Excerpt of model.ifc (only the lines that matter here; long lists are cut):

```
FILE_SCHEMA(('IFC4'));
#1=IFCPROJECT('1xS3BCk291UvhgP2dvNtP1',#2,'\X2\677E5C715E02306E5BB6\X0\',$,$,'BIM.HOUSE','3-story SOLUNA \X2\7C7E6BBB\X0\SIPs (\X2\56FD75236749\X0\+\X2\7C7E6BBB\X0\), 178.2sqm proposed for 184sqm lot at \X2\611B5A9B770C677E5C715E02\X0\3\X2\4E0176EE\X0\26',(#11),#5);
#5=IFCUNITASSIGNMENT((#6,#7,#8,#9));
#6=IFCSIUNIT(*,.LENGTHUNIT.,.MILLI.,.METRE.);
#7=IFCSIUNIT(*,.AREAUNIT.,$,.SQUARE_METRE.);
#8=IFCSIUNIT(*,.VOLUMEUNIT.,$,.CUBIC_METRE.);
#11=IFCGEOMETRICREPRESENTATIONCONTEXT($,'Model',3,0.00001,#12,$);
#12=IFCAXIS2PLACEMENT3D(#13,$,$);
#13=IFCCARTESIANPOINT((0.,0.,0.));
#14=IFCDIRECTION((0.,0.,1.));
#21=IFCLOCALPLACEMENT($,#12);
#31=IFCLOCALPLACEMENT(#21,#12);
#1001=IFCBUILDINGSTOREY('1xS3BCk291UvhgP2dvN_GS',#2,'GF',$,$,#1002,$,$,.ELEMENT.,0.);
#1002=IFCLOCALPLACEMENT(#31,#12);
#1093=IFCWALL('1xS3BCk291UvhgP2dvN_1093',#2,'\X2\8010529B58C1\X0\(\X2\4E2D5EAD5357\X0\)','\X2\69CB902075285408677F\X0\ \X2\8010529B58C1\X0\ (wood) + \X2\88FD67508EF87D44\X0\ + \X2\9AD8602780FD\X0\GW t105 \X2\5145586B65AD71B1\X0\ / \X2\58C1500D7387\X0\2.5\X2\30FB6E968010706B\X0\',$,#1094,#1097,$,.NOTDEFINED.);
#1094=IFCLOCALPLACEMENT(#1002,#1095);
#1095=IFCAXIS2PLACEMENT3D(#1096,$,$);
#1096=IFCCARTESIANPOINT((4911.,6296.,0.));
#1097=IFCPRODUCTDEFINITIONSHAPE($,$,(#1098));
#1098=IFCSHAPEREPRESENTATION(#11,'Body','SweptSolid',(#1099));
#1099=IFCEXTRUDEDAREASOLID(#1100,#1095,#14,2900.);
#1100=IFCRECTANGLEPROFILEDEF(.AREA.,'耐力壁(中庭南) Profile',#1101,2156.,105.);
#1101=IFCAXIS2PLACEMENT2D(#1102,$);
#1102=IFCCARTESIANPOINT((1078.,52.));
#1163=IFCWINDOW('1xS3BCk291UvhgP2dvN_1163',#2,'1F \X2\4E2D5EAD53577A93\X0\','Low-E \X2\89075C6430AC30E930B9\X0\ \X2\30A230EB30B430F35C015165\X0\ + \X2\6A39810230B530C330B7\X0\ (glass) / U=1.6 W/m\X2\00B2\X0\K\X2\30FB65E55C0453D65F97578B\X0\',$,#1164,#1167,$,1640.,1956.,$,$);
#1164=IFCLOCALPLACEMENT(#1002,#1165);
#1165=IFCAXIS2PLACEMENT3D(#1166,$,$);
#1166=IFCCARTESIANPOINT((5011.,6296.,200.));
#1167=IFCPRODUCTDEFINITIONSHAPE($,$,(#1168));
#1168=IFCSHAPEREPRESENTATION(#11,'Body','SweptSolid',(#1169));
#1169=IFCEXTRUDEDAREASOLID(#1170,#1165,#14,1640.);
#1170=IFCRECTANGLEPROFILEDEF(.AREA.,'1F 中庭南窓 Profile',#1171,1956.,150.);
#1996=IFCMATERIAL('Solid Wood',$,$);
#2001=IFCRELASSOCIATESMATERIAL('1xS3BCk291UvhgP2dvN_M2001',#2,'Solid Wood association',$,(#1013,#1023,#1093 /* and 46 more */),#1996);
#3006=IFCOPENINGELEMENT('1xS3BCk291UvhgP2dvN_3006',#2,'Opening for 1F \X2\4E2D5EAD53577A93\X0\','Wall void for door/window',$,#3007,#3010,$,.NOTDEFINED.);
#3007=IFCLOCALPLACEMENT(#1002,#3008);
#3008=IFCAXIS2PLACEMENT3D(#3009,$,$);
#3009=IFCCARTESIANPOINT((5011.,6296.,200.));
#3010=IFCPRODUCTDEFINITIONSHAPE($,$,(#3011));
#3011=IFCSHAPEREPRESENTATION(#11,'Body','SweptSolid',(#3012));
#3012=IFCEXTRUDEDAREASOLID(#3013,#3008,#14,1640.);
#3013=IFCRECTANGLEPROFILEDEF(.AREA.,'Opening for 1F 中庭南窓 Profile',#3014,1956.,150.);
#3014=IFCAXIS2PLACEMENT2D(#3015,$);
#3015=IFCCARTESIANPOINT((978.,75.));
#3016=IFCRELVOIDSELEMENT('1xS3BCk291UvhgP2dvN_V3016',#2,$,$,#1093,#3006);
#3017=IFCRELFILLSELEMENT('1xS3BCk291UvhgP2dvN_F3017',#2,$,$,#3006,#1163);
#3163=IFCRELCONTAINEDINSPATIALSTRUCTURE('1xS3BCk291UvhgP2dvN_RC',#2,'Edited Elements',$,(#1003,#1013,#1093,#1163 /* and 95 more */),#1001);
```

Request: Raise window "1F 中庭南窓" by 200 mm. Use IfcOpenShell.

```python
import numpy as np
import ifcopenshell
import ifcopenshell.api.geometry
import ifcopenshell.util.placement
import ifcopenshell.util.unit

model = ifcopenshell.open("model.ifc")
unit_scale = ifcopenshell.util.unit.calculate_unit_scale(model)

window = model.by_guid("1xS3BCk291UvhgP2dvN_1163")
opening = window.FillsVoids[0].RelatingOpeningElement
dz = 0.2 / unit_scale

shift = np.array([0.0, 0.0, dz])
# The window is not placed relative to its opening, so move both.
for product in (opening, window):
    matrix = ifcopenshell.util.placement.get_local_placement(product.ObjectPlacement)
    matrix[:3, 3] += shift
    ifcopenshell.api.geometry.edit_object_placement(model, product=product, matrix=matrix, is_si=False)

print(f"moved by {dz * unit_scale:+.3f} m")

model.write("model-out.ifc")
```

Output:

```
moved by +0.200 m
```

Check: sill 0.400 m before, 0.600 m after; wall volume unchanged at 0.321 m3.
